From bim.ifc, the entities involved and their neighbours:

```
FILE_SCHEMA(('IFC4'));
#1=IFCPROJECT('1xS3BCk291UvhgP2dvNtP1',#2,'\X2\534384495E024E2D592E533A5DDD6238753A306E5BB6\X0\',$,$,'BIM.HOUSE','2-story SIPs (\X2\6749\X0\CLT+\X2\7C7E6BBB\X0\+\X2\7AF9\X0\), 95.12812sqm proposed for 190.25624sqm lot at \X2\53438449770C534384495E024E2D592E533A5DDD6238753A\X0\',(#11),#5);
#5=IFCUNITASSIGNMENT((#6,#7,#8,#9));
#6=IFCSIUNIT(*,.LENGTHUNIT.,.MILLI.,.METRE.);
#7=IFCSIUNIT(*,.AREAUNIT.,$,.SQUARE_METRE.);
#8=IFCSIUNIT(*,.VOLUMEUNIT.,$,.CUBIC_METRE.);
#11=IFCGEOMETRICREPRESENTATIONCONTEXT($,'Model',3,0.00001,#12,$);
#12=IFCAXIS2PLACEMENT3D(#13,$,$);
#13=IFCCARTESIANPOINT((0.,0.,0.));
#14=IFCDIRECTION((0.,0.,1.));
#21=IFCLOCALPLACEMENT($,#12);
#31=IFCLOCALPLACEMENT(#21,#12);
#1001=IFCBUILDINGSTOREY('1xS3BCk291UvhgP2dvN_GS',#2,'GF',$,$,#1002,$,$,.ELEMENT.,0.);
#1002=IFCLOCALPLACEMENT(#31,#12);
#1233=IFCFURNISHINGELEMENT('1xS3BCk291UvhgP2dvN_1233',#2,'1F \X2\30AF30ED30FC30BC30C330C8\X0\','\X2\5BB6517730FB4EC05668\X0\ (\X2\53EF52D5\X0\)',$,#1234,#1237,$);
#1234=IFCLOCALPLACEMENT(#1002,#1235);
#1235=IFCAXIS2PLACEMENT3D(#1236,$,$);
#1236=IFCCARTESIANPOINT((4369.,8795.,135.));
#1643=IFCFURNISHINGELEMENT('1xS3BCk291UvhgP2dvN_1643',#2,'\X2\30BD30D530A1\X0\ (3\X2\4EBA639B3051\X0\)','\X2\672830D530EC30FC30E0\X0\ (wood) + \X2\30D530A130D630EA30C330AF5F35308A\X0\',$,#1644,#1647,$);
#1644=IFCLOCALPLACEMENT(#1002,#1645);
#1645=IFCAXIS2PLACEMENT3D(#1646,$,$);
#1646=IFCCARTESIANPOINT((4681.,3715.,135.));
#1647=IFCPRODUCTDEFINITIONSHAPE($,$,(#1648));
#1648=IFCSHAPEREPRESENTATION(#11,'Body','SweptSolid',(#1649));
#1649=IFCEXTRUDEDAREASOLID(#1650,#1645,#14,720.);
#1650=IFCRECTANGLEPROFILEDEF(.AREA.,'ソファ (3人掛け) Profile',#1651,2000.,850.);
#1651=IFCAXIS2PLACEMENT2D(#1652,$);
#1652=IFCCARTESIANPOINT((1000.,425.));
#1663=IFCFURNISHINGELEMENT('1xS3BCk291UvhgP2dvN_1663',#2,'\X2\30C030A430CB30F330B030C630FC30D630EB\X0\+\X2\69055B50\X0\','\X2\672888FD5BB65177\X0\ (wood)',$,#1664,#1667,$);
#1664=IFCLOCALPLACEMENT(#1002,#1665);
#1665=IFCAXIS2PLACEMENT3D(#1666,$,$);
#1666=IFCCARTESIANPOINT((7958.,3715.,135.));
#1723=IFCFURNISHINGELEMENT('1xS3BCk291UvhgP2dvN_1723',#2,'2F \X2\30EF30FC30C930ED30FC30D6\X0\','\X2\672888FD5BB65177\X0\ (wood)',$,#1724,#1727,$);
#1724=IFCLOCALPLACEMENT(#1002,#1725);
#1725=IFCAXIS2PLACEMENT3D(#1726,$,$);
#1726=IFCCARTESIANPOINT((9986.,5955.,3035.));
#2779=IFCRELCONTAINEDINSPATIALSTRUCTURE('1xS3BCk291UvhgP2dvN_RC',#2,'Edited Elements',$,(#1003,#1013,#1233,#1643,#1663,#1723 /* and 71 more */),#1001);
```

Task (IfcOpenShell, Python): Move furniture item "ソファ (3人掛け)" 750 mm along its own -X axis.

```python
import ifcopenshell
import ifcopenshell.api.geometry
import ifcopenshell.util.placement
import ifcopenshell.util.unit

model = ifcopenshell.open("bim.ifc")
unit_scale = ifcopenshell.util.unit.calculate_unit_scale(model)

item = model.by_guid("1xS3BCk291UvhgP2dvN_1643")
matrix = ifcopenshell.util.placement.get_local_placement(item.ObjectPlacement)
matrix[:3, 3] -= matrix[:3, 0] * 0.75 / unit_scale
ifcopenshell.api.geometry.edit_object_placement(model, product=item, matrix=matrix, is_si=False)

print(ifcopenshell.util.placement.get_local_placement(item.ObjectPlacement).round(3) + 0.0)

model.write("bim_edited.ifc")
```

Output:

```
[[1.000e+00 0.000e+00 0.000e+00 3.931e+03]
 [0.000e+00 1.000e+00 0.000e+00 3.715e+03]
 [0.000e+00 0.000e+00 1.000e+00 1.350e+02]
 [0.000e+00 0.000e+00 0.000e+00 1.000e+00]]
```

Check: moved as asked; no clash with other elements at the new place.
